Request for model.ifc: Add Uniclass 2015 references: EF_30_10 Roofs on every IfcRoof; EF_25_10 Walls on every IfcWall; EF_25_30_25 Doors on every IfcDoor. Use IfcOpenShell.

First a look at what the model holds.

```python
import ifcopenshell

model = ifcopenshell.open("model.ifc")
print(model.schema)
print("classifications:", [c.Name for c in model.by_type("IfcClassification")])
for ifc_class in ("IfcDoor", "IfcRoof", "IfcStair", "IfcWall", "IfcWindow"):
    print(ifc_class, len(model.by_type(ifc_class)))
```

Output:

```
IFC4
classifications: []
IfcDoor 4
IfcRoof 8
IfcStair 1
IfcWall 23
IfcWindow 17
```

```python
import ifcopenshell
import ifcopenshell.api.classification

model = ifcopenshell.open("model.ifc")

system = ifcopenshell.api.classification.add_classification(model, classification="Uniclass 2015")

codes = {
    "IfcRoof": ("EF_30_10", "Roofs"),
    "IfcWall": ("EF_25_10", "Walls"),
    "IfcDoor": ("EF_25_30_25", "Doors"),
}
for ifc_class, (code, name) in codes.items():
    products = model.by_type(ifc_class)
    ifcopenshell.api.classification.add_reference(
        model, products=products, classification=system, identification=code, name=name
    )
    print(code, len(products))

model.write("model_rev.ifc")
```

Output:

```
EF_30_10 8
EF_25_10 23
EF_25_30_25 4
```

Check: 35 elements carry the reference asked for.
